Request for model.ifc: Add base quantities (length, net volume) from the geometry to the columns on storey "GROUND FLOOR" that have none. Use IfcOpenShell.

First a look at what the model holds.

```python
import ifcopenshell
import ifcopenshell.util.element
import ifcopenshell.util.unit

model = ifcopenshell.open("model.ifc")
print(model.schema)
for unit_type in ("LENGTHUNIT", "AREAUNIT", "VOLUMEUNIT"):
    print(unit_type, ifcopenshell.util.unit.calculate_unit_scale(model, unit_type))
storey = next(s for s in model.by_type("IfcBuildingStorey") if s.Name == "GROUND FLOOR")
columns = [e for e in ifcopenshell.util.element.get_decomposition(storey) if e.is_a("IfcColumn")]
for e in sorted(columns, key=lambda e: e.id()):
    print(e.id(), e.is_a(), e.Name, list(ifcopenshell.util.element.get_psets(e, qtos_only=True)), sep=" | ")
```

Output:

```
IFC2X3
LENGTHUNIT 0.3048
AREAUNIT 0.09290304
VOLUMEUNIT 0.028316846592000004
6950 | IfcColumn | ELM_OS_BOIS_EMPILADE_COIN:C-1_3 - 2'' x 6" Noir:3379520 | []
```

```python
import ifcopenshell
import ifcopenshell.api.pset
import ifcopenshell.geom
import ifcopenshell.util.element
import ifcopenshell.util.shape
import ifcopenshell.util.unit

model = ifcopenshell.open("model.ifc")
unit_scale = ifcopenshell.util.unit.calculate_unit_scale(model)
volume_scale = ifcopenshell.util.unit.calculate_unit_scale(model, "VOLUMEUNIT")
settings = ifcopenshell.geom.settings()

storey = next(s for s in model.by_type("IfcBuildingStorey") if s.Name == "GROUND FLOOR")
columns = [e for e in ifcopenshell.util.element.get_decomposition(storey) if e.is_a("IfcColumn")]

for e in sorted(columns, key=lambda e: e.id()):
    if ifcopenshell.util.element.get_psets(e, qtos_only=True, should_inherit=False):
        continue
    # Geometry comes back in metres, in the element's own axes.
    shape = ifcopenshell.geom.create_shape(settings, e)
    values = {
        "Length": ifcopenshell.util.shape.get_z(shape.geometry) / unit_scale,
        "NetVolume": ifcopenshell.util.shape.get_volume(shape.geometry) / volume_scale,
    }
    qto = ifcopenshell.api.pset.add_qto(model, product=e, name="BaseQuantities")
    ifcopenshell.api.pset.edit_qto(model, qto=qto, properties=values)
    print(e.id(), {k: round(v, 3) for k, v in values.items()})

model.write("model_rev.ifc")
```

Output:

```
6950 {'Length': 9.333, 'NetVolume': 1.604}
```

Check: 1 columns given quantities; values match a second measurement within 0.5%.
